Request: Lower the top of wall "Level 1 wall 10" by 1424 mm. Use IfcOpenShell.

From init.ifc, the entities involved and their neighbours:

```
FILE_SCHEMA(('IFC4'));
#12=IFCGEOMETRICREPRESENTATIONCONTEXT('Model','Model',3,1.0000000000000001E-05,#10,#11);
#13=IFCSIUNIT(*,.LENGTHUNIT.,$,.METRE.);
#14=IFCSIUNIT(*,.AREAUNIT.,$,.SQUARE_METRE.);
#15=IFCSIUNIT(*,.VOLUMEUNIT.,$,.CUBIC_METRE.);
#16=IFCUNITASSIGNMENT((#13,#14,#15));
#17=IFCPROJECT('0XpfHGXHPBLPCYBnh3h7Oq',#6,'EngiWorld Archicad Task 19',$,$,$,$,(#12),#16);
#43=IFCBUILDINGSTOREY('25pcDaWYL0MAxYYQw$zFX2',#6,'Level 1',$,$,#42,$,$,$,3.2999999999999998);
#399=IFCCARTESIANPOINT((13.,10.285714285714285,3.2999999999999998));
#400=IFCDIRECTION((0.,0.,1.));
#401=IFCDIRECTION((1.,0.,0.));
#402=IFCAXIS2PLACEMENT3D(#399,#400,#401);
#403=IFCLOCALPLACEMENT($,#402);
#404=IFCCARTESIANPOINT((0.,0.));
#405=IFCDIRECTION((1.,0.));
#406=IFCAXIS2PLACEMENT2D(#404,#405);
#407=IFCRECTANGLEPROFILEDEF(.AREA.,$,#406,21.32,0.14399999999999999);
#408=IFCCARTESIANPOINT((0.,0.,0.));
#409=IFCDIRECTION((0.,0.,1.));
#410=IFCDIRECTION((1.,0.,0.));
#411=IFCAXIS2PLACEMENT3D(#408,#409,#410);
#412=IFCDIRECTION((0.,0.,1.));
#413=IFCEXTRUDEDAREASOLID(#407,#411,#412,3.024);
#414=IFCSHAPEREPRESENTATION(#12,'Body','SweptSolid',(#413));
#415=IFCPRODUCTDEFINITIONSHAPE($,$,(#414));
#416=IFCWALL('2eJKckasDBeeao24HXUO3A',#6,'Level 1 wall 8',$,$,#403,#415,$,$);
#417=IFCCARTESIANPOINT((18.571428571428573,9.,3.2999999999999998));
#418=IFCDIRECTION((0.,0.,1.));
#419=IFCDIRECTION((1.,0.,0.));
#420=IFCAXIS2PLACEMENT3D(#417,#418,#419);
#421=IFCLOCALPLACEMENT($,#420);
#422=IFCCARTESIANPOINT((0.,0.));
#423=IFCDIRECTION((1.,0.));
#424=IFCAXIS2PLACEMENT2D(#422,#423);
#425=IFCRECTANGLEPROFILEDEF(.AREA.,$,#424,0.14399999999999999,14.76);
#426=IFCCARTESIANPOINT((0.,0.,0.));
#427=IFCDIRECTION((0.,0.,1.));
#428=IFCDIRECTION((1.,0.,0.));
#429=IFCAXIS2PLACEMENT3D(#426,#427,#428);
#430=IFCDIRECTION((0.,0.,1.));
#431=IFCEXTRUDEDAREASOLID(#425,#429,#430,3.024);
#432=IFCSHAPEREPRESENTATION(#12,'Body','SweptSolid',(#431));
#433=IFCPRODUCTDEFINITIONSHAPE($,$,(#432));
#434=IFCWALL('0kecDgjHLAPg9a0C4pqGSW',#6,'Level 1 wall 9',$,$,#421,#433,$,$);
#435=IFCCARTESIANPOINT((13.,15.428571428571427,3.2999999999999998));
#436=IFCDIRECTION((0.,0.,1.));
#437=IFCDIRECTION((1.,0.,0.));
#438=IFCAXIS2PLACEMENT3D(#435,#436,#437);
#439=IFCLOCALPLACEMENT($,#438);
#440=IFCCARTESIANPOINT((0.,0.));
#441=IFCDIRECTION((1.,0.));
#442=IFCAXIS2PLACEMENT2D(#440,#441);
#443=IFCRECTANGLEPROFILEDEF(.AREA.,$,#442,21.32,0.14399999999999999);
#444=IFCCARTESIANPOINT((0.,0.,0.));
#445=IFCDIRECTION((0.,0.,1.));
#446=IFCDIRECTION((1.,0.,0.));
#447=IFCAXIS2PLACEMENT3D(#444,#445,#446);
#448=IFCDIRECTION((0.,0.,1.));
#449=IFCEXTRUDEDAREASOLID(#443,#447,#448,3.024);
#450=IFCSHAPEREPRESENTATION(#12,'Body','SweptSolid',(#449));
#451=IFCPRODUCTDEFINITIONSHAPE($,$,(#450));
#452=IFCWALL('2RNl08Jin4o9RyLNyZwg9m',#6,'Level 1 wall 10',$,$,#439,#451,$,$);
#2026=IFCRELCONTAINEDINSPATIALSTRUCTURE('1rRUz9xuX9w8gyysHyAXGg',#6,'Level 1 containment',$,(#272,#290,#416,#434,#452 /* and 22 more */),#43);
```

```python
import ifcopenshell
import ifcopenshell.geom
import ifcopenshell.util.shape
import ifcopenshell.util.unit

model = ifcopenshell.open("init.ifc")
unit_scale = ifcopenshell.util.unit.calculate_unit_scale(model)
settings = ifcopenshell.geom.settings()


def volume(element):
    """Net volume in cubic metres, openings subtracted."""
    shape = ifcopenshell.geom.create_shape(settings, element)
    return ifcopenshell.util.shape.get_volume(shape.geometry)


wall = model.by_id(452)
before = volume(wall)

body = next(r for r in wall.Representation.Representations if r.RepresentationIdentifier == "Body")
solid = body.Items[0]
old_height = solid.Depth
solid.Depth -= 1.424 / unit_scale
after = volume(wall)

print(f"height {old_height:g} -> {solid.Depth:g}, volume {before:.3f} -> {after:.3f} m3")

model.write("init_v2.ifc")
```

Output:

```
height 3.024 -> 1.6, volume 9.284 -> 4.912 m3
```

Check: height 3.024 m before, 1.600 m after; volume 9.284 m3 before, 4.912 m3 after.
